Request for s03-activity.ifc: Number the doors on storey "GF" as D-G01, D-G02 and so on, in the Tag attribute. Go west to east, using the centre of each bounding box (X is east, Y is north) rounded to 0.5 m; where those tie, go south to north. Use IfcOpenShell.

First a look at what the model holds.

```python
import ifcopenshell
import ifcopenshell.util.element
import ifcopenshell.util.placement

model = ifcopenshell.open("s03-activity.ifc")
print(model.schema)
storey = next(s for s in model.by_type("IfcBuildingStorey") if s.Name == "GF")
doors = [e for e in ifcopenshell.util.element.get_decomposition(storey) if e.is_a("IfcDoor")]
for e in sorted(doors, key=lambda e: e.id()):
    origin = ifcopenshell.util.placement.get_local_placement(e.ObjectPlacement)[:3, 3]
    print(e.id(), e.Tag, e.Name, origin.round(2) + 0.0, sep=" | ")
```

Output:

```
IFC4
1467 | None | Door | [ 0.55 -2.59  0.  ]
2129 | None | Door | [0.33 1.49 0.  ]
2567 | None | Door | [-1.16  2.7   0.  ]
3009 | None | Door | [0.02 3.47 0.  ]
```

```python
import ifcopenshell
import ifcopenshell.geom
import ifcopenshell.util.element
import ifcopenshell.util.shape

model = ifcopenshell.open("s03-activity.ifc")
settings = ifcopenshell.geom.settings()
settings.set("use-world-coords", True)


def centre(element):
    shape = ifcopenshell.geom.create_shape(settings, element)
    return ifcopenshell.util.shape.get_bbox_centroid(shape.geometry)


storey = next(s for s in model.by_type("IfcBuildingStorey") if s.Name == "GF")
doors = [e for e in ifcopenshell.util.element.get_decomposition(storey) if e.is_a("IfcDoor")]

# Insertion points can sit at a corner or the storey origin, so sort by the geometry (in metres).
centres = {e: centre(e) for e in doors}
doors.sort(key=lambda e: (round(centres[e][0] / 0.5), centres[e][1]))

for i, e in enumerate(doors, start=1):
    number = f"D-G{i:02d}"
    e.Tag = number
    print(e.id(), number)

model.write("s03-activity_edited.ifc")
```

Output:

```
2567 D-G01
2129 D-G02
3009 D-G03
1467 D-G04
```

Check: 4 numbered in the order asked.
